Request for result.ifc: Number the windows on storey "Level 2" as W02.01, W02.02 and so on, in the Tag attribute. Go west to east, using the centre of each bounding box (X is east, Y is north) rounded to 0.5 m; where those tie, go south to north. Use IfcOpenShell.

First a look at what the model holds.

```python
import ifcopenshell
import ifcopenshell.util.element
import ifcopenshell.util.placement

model = ifcopenshell.open("result.ifc")
print(model.schema)
storey = next(s for s in model.by_type("IfcBuildingStorey") if s.Name == "Level 2")
windows = [e for e in ifcopenshell.util.element.get_decomposition(storey) if e.is_a("IfcWindow")]
for e in sorted(windows, key=lambda e: e.id()):
    origin = ifcopenshell.util.placement.get_local_placement(e.ObjectPlacement)[:3, 3]
    print(e.id(), e.Tag, e.Name, origin.round(2) + 0.0, sep=" | ")
```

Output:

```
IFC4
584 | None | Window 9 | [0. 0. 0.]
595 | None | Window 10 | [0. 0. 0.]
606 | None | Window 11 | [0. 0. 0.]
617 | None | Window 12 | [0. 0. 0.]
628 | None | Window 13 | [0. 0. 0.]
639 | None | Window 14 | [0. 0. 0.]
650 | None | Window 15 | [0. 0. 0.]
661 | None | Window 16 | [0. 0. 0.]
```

```python
import ifcopenshell
import ifcopenshell.geom
import ifcopenshell.util.element
import ifcopenshell.util.shape

model = ifcopenshell.open("result.ifc")
settings = ifcopenshell.geom.settings()
settings.set("use-world-coords", True)


def centre(element):
    shape = ifcopenshell.geom.create_shape(settings, element)
    return ifcopenshell.util.shape.get_bbox_centroid(shape.geometry)


storey = next(s for s in model.by_type("IfcBuildingStorey") if s.Name == "Level 2")
windows = [e for e in ifcopenshell.util.element.get_decomposition(storey) if e.is_a("IfcWindow")]

# Insertion points can sit at a corner or the storey origin, so sort by the geometry (in metres).
centres = {e: centre(e) for e in windows}
windows.sort(key=lambda e: (round(centres[e][0] / 0.5), centres[e][1]))

for i, e in enumerate(windows, start=1):
    number = f"W02.{i:02d}"
    e.Tag = number
    print(e.id(), number)

model.write("result_v2.ifc")
```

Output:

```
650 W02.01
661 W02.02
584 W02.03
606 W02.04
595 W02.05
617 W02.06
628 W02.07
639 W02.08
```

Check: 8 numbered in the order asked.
